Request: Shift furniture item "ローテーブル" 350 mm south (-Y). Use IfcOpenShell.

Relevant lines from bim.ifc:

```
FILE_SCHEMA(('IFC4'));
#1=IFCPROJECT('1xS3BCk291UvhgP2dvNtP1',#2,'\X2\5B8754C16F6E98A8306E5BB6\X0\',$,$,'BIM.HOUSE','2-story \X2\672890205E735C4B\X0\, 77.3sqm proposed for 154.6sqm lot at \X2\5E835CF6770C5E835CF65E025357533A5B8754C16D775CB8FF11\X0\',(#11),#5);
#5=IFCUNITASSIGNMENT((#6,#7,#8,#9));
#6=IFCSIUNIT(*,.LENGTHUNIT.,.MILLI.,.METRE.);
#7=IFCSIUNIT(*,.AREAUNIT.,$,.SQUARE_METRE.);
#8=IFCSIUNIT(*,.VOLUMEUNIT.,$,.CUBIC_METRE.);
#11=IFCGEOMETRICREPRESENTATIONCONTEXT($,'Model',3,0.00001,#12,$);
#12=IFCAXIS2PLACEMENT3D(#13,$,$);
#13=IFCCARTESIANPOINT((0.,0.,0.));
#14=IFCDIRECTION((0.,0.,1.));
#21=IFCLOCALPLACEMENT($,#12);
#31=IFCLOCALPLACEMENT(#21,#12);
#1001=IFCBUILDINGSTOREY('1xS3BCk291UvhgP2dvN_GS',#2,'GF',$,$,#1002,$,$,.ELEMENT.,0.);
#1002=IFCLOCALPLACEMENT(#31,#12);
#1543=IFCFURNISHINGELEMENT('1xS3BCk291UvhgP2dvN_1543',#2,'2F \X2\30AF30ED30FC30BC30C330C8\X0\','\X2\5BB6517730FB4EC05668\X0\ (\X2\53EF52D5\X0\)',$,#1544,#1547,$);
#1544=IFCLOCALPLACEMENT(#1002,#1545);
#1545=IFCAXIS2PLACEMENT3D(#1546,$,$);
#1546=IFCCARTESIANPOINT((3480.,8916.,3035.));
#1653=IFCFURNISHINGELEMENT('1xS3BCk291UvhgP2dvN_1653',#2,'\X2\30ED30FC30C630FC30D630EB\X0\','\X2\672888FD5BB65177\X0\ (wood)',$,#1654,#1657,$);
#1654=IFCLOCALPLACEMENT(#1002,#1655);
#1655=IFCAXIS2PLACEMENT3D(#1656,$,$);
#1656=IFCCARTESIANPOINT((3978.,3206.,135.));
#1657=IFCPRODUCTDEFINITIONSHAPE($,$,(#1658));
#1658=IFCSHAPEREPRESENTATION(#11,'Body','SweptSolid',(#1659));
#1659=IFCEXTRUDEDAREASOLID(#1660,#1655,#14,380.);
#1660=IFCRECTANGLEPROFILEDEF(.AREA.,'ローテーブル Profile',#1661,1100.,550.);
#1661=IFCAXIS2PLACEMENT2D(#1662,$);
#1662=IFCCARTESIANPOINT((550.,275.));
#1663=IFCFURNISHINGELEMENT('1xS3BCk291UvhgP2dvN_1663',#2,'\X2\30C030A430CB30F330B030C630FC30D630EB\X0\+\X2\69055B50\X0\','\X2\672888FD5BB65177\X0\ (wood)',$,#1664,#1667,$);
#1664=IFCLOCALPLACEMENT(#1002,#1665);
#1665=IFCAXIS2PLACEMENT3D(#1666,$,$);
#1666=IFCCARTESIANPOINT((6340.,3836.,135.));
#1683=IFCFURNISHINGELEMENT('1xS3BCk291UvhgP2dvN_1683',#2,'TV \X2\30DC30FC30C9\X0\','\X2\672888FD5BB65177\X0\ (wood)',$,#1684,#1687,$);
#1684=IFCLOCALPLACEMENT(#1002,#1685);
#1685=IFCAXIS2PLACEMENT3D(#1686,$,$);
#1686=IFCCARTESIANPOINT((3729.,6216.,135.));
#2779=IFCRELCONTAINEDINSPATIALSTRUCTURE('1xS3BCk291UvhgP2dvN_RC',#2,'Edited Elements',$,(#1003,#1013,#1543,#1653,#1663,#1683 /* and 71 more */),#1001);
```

```python
import ifcopenshell
import ifcopenshell.api.geometry
import ifcopenshell.util.placement
import ifcopenshell.util.unit

model = ifcopenshell.open("bim.ifc")
unit_scale = ifcopenshell.util.unit.calculate_unit_scale(model)

item = model.by_id(1653)
matrix = ifcopenshell.util.placement.get_local_placement(item.ObjectPlacement)
matrix[1, 3] -= 0.35 / unit_scale
ifcopenshell.api.geometry.edit_object_placement(model, product=item, matrix=matrix, is_si=False)

print(ifcopenshell.util.placement.get_local_placement(item.ObjectPlacement).round(3) + 0.0)

model.write("bim_rev.ifc")
```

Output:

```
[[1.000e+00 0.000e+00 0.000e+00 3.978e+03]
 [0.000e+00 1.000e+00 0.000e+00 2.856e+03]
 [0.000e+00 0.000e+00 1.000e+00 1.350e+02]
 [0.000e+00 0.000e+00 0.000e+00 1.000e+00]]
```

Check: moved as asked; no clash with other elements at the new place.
